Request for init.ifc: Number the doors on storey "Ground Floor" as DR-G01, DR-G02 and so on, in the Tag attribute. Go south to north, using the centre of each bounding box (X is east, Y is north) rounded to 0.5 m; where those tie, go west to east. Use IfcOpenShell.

First a look at what the model holds.

```python
import ifcopenshell
import ifcopenshell.util.element
import ifcopenshell.util.placement

model = ifcopenshell.open("init.ifc")
print(model.schema)
storey = next(s for s in model.by_type("IfcBuildingStorey") if s.Name == "Ground Floor")
doors = [e for e in ifcopenshell.util.element.get_decomposition(storey) if e.is_a("IfcDoor")]
for e in sorted(doors, key=lambda e: e.id()):
    origin = ifcopenshell.util.placement.get_local_placement(e.ObjectPlacement)[:3, 3]
    print(e.id(), e.Tag, e.Name, origin.round(2) + 0.0, sep=" | ")
```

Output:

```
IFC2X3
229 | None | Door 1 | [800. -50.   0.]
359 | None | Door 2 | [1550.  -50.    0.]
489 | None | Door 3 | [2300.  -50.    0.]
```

```python
import ifcopenshell
import ifcopenshell.geom
import ifcopenshell.util.element
import ifcopenshell.util.shape

model = ifcopenshell.open("init.ifc")
settings = ifcopenshell.geom.settings()
settings.set("use-world-coords", True)


def centre(element):
    shape = ifcopenshell.geom.create_shape(settings, element)
    return ifcopenshell.util.shape.get_bbox_centroid(shape.geometry)


storey = next(s for s in model.by_type("IfcBuildingStorey") if s.Name == "Ground Floor")
doors = [e for e in ifcopenshell.util.element.get_decomposition(storey) if e.is_a("IfcDoor")]

# Insertion points can sit at a corner or the storey origin, so sort by the geometry (in metres).
centres = {e: centre(e) for e in doors}
doors.sort(key=lambda e: (round(centres[e][1] / 0.5), centres[e][0]))

for i, e in enumerate(doors, start=1):
    number = f"DR-G{i:02d}"
    e.Tag = number
    print(e.id(), number)

model.write("init_v2.ifc")
```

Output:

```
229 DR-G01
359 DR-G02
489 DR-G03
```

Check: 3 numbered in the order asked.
